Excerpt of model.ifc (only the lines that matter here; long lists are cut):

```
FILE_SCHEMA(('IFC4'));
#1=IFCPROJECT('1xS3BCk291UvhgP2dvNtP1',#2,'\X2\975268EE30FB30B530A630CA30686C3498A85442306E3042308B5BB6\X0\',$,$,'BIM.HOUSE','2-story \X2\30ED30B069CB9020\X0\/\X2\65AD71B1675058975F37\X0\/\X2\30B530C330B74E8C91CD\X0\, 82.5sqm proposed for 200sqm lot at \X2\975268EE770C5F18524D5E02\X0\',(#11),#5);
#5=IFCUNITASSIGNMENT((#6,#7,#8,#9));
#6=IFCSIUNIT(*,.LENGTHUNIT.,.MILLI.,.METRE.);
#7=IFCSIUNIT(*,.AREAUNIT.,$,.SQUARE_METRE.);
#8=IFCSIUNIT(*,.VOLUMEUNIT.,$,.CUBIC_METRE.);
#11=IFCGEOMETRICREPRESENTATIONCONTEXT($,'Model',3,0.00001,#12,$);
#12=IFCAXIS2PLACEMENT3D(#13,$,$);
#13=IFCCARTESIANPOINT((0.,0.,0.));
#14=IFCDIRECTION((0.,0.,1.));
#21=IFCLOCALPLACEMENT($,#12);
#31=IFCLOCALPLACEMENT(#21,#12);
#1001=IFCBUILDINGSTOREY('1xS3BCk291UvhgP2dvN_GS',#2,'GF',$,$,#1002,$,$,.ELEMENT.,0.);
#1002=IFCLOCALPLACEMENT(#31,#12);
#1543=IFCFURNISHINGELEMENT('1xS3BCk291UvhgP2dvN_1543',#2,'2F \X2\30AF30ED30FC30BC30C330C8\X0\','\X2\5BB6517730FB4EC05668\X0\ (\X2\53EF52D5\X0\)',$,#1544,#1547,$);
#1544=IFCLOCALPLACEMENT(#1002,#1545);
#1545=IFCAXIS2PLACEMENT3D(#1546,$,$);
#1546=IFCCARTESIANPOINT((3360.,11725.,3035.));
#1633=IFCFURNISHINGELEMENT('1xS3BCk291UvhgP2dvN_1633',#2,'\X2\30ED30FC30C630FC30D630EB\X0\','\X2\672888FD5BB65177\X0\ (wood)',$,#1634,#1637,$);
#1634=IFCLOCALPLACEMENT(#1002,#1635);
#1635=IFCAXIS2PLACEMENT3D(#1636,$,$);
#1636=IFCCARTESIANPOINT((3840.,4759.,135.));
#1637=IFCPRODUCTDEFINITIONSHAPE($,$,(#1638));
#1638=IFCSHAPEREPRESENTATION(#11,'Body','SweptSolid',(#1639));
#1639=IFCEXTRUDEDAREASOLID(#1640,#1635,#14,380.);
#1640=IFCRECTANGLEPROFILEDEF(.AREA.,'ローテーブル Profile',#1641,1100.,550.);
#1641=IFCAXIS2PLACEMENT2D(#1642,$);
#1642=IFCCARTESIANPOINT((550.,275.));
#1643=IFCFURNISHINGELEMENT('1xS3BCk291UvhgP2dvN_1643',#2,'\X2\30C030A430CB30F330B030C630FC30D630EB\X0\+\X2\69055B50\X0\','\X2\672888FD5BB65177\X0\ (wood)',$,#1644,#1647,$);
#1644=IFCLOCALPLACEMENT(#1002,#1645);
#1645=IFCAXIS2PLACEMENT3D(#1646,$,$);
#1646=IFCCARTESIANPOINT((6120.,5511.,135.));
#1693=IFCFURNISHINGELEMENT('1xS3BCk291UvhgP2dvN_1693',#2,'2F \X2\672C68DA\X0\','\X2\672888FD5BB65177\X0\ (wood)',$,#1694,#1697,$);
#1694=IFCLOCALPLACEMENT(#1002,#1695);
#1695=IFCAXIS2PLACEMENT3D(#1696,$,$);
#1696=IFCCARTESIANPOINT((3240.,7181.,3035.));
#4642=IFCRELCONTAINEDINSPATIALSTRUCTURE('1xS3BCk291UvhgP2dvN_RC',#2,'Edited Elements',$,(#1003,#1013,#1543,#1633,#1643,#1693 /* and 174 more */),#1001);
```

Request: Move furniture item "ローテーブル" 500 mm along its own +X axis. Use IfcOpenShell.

```python
import ifcopenshell
import ifcopenshell.api.geometry
import ifcopenshell.util.placement

model = ifcopenshell.open("model.ifc")

item = model.by_id(1633)
matrix = ifcopenshell.util.placement.get_local_placement(item.ObjectPlacement)
matrix[:3, 3] += matrix[:3, 0] * 500.0
ifcopenshell.api.geometry.edit_object_placement(model, product=item, matrix=matrix, is_si=False)

print(ifcopenshell.util.placement.get_local_placement(item.ObjectPlacement).round(3) + 0.0)

model.write("model_edited.ifc")
```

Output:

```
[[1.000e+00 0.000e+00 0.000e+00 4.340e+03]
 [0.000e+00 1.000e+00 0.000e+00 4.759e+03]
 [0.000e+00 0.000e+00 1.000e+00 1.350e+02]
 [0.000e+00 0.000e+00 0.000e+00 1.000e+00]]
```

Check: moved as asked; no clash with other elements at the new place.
